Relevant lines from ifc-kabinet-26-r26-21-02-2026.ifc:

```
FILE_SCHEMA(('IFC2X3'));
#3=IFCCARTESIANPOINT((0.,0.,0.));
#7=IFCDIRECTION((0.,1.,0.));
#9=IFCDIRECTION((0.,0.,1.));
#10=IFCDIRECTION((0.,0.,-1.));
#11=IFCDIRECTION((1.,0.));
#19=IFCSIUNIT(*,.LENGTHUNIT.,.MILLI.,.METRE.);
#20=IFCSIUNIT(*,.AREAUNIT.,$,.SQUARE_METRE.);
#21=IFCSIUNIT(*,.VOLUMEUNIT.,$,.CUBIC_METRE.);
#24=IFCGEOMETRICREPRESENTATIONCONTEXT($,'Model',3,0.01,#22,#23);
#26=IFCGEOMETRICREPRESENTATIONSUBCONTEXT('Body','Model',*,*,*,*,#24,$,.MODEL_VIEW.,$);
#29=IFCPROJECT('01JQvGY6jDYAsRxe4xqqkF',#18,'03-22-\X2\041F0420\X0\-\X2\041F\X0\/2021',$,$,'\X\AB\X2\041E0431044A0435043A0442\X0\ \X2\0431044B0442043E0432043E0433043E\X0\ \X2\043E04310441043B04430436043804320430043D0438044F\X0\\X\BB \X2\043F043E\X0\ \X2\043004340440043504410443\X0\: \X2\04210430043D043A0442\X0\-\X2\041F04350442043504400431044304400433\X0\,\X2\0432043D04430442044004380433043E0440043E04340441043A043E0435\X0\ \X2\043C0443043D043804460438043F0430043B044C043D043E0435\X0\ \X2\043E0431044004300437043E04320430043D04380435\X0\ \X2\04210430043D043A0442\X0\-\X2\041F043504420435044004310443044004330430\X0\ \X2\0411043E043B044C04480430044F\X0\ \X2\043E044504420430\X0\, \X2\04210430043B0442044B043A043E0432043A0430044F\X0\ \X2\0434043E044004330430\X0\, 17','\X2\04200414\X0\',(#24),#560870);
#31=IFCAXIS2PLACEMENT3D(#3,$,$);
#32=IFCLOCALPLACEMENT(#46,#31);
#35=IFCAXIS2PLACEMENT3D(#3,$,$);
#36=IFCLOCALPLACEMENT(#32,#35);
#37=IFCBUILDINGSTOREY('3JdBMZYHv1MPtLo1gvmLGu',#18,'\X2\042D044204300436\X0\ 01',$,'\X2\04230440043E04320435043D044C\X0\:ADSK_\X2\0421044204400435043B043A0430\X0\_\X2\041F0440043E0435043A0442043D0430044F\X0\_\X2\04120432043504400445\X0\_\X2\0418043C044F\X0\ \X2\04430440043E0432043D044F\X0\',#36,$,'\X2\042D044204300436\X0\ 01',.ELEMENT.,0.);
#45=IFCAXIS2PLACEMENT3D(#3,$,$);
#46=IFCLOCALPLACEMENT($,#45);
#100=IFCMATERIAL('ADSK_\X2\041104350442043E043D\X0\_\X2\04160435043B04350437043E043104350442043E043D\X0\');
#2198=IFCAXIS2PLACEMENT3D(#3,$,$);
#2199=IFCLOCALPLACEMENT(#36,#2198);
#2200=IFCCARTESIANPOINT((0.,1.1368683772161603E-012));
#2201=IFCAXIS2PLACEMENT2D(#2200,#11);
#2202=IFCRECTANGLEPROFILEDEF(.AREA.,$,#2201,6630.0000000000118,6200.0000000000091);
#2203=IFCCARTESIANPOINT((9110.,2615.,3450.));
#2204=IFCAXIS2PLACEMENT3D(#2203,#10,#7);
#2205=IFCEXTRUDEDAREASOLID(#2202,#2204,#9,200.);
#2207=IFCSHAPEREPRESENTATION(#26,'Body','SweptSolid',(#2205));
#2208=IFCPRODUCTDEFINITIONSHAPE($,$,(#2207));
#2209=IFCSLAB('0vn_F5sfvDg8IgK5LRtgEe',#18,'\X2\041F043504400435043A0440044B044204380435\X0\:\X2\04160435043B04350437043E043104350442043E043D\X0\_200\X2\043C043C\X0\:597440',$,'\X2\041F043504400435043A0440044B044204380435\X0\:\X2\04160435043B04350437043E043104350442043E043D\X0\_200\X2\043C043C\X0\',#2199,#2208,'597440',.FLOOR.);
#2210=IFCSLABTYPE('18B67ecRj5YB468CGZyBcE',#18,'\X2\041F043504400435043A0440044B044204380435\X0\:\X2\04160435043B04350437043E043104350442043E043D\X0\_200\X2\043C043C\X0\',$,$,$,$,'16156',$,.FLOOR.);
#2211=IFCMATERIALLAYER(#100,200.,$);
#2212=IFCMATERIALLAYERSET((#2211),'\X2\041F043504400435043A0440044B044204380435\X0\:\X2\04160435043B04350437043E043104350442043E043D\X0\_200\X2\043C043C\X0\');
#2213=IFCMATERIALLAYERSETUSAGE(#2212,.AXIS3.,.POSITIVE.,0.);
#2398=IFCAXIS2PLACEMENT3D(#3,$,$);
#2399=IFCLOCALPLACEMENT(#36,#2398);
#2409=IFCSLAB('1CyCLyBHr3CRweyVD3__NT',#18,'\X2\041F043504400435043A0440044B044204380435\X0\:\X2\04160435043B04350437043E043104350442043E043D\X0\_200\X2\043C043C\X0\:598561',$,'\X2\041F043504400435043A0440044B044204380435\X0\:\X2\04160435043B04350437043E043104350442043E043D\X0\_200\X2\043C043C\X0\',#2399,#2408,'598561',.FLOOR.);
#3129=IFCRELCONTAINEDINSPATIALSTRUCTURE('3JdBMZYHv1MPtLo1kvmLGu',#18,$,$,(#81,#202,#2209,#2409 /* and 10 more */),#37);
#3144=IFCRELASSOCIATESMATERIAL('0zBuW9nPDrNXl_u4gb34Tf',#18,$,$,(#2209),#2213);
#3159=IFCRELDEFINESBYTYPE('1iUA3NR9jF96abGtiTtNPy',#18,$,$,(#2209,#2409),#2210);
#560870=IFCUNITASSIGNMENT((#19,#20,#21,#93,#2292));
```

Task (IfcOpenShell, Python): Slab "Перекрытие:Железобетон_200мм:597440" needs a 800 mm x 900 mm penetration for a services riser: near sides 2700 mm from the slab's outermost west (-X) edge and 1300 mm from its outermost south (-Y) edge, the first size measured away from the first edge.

```python
import numpy as np
import ifcopenshell
import ifcopenshell.api.feature
import ifcopenshell.api.geometry
import ifcopenshell.api.root
import ifcopenshell.geom
import ifcopenshell.util.placement
import ifcopenshell.util.representation
import ifcopenshell.util.shape
import ifcopenshell.util.unit

model = ifcopenshell.open("ifc-kabinet-26-r26-21-02-2026.ifc")
unit_scale = ifcopenshell.util.unit.calculate_unit_scale(model)
settings = ifcopenshell.geom.settings()


def volume(element):
    """Net volume in cubic metres, openings subtracted."""
    shape = ifcopenshell.geom.create_shape(settings, element)
    return ifcopenshell.util.shape.get_volume(shape.geometry)


slab = model.by_guid("0vn_F5sfvDg8IgK5LRtgEe")
before = volume(slab)

# Extent in the slab's own axes, in metres. The edges named are its -X and -Y sides.
slab_shape = ifcopenshell.geom.create_shape(settings, slab)
vertices = ifcopenshell.util.shape.get_vertices(slab_shape.geometry)
x_min, y_min, bottom = vertices.min(axis=0)
top = vertices[:, 2].max()

opening = ifcopenshell.api.root.create_entity(model, ifc_class="IfcOpeningElement", name="Services riser opening")
context = ifcopenshell.util.representation.get_context(model, "Model", "Body", "MODEL_VIEW")
width, depth = 0.8, 0.9
outline = [(0.0, 0.0), (width, 0.0), (width, depth), (0.0, depth), (0.0, 0.0)]
# Overshoot both faces by 50 mm so the cut is clean.
shape = ifcopenshell.api.geometry.add_slab_representation(
    model, context=context, depth=top - bottom + 0.1, polyline=outline
)
ifcopenshell.api.geometry.assign_representation(model, product=opening, representation=shape)

matrix = ifcopenshell.util.placement.get_local_placement(slab.ObjectPlacement)
matrix[:, 3] = matrix @ np.append(np.array([x_min + 2.7, y_min + 1.3, bottom - 0.05]) / unit_scale, 1.0)
ifcopenshell.api.geometry.edit_object_placement(model, product=opening, matrix=matrix, is_si=False)
ifcopenshell.api.feature.add_feature(model, feature=opening, element=slab)

after = volume(slab)

print(f"slab volume {before:.3f} -> {after:.3f} m3")

model.write("ifc-kabinet-26-r26-21-02-2026_updated.ifc")
```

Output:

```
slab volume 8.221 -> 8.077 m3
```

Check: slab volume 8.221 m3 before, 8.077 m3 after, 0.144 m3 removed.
